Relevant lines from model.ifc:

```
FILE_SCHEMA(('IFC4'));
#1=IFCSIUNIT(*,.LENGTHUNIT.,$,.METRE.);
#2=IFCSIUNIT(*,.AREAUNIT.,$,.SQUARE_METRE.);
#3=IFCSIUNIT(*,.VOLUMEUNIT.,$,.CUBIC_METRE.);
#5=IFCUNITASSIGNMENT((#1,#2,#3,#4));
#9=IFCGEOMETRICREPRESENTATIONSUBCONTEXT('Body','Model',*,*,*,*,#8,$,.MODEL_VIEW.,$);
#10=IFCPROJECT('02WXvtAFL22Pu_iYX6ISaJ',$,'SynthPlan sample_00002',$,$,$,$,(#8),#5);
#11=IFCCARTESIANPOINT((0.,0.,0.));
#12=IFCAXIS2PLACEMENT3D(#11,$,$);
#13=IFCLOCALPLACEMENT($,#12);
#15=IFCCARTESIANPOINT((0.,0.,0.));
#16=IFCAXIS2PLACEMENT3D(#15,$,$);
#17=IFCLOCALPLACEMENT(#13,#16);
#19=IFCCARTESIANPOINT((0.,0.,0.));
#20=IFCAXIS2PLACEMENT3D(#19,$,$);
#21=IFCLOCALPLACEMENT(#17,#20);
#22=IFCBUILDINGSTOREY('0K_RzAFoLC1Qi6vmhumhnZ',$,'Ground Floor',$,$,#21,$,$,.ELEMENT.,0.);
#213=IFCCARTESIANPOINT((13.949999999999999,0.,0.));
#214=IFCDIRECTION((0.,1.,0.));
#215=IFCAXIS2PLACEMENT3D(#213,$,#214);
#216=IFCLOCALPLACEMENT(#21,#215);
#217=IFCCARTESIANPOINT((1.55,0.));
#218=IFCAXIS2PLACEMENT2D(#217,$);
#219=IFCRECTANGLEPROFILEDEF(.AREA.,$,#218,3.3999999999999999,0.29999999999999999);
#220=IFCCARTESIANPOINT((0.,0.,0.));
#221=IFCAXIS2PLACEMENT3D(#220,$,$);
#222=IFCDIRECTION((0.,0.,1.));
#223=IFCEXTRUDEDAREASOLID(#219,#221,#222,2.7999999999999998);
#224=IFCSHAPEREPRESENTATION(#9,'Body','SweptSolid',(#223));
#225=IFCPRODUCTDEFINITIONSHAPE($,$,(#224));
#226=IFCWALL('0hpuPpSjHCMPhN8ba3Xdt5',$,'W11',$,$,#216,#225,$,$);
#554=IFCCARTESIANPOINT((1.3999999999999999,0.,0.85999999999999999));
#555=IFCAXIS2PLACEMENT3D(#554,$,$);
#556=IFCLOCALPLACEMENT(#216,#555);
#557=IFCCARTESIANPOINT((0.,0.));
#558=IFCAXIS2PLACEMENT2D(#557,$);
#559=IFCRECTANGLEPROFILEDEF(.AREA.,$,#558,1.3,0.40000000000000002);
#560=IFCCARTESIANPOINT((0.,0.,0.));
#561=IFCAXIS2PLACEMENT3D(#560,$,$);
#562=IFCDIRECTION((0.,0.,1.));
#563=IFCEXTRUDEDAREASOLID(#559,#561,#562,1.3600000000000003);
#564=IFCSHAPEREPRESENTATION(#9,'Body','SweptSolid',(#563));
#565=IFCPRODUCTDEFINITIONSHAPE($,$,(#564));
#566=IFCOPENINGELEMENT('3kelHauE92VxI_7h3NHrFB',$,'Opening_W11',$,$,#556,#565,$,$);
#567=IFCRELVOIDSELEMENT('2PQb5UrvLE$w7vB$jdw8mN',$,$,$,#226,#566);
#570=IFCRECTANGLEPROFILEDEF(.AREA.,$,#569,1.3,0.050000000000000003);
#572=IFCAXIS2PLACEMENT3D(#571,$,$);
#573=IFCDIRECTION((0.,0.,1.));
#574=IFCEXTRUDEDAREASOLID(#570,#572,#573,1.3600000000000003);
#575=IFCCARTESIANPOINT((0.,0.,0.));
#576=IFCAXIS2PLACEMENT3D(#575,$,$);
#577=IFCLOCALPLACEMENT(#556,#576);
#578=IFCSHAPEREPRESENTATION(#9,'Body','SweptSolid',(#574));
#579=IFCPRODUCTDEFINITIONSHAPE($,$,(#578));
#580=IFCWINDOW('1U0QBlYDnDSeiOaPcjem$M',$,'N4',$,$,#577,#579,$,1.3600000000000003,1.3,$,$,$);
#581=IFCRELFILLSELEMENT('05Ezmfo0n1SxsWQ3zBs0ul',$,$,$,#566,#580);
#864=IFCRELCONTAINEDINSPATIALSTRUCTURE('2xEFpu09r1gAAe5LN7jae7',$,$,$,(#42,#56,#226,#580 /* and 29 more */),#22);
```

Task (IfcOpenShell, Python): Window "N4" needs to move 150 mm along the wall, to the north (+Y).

```python
import ifcopenshell
import ifcopenshell.api.geometry
import ifcopenshell.util.placement
import ifcopenshell.util.unit

model = ifcopenshell.open("model.ifc")
unit_scale = ifcopenshell.util.unit.calculate_unit_scale(model)

window = model.by_guid("1U0QBlYDnDSeiOaPcjem$M")
opening = window.FillsVoids[0].RelatingOpeningElement
wall = opening.VoidsElements[0].RelatingBuildingElement

wall_matrix = ifcopenshell.util.placement.get_local_placement(wall.ObjectPlacement)
shift = wall_matrix[:3, 0] * 0.15 / unit_scale
before = ifcopenshell.util.placement.get_local_placement(window.ObjectPlacement)[:3, 3].copy()

# The window is placed relative to its opening, so it follows when the opening moves.
matrix = ifcopenshell.util.placement.get_local_placement(opening.ObjectPlacement)
matrix[:3, 3] += shift
ifcopenshell.api.geometry.edit_object_placement(
    model, product=opening, matrix=matrix, is_si=False, should_transform_children=True
)

after = ifcopenshell.util.placement.get_local_placement(window.ObjectPlacement)[:3, 3]
print("window moved by", (after - before).round(3) + 0.0)

model.write("model-out.ifc")
```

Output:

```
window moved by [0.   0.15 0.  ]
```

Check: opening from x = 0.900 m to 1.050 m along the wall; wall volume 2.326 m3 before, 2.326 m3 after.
